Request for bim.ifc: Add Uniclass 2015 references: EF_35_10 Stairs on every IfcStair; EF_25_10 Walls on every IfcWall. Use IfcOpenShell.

First a look at what the model holds.

```python
import ifcopenshell

model = ifcopenshell.open("bim.ifc")
print(model.schema)
print("classifications:", [c.Name for c in model.by_type("IfcClassification")])
for ifc_class in ("IfcDoor", "IfcRoof", "IfcStair", "IfcWall", "IfcWindow"):
    print(ifc_class, len(model.by_type(ifc_class)))
```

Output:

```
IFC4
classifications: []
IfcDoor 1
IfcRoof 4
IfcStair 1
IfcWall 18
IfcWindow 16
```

```python
import ifcopenshell
import ifcopenshell.api.classification

model = ifcopenshell.open("bim.ifc")

system = ifcopenshell.api.classification.add_classification(model, classification="Uniclass 2015")

codes = {
    "IfcStair": ("EF_35_10", "Stairs"),
    "IfcWall": ("EF_25_10", "Walls"),
}
for ifc_class, (code, name) in codes.items():
    products = model.by_type(ifc_class)
    ifcopenshell.api.classification.add_reference(
        model, products=products, classification=system, identification=code, name=name
    )
    print(code, len(products))

model.write("bim-out.ifc")
```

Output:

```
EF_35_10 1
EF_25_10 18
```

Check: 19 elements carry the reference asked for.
